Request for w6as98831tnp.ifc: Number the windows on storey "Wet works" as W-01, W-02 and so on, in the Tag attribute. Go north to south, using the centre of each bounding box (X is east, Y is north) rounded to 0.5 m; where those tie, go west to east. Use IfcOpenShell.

First a look at what the model holds.

```python
import ifcopenshell
import ifcopenshell.util.element
import ifcopenshell.util.placement

model = ifcopenshell.open("w6as98831tnp.ifc")
print(model.schema)
storey = next(s for s in model.by_type("IfcBuildingStorey") if s.Name == "Wet works")
windows = [e for e in ifcopenshell.util.element.get_decomposition(storey) if e.is_a("IfcWindow")]
for e in sorted(windows, key=lambda e: e.id()):
    origin = ifcopenshell.util.placement.get_local_placement(e.ObjectPlacement)[:3, 3]
    print(e.id(), e.Tag, e.Name, origin.round(2) + 0.0, sep=" | ")
```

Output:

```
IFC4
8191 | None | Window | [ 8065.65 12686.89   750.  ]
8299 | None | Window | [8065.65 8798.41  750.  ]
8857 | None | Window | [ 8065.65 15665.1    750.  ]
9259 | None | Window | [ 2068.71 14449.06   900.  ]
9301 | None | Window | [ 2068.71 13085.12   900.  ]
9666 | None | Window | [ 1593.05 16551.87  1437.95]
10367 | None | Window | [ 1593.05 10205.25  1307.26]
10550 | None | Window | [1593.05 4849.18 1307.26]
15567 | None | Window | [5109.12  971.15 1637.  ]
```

```python
import ifcopenshell
import ifcopenshell.geom
import ifcopenshell.util.element
import ifcopenshell.util.shape

model = ifcopenshell.open("w6as98831tnp.ifc")
settings = ifcopenshell.geom.settings()
settings.set("use-world-coords", True)


def centre(element):
    shape = ifcopenshell.geom.create_shape(settings, element)
    return ifcopenshell.util.shape.get_bbox_centroid(shape.geometry)


storey = next(s for s in model.by_type("IfcBuildingStorey") if s.Name == "Wet works")
windows = [e for e in ifcopenshell.util.element.get_decomposition(storey) if e.is_a("IfcWindow")]

# Insertion points can sit at a corner or the storey origin, so sort by the geometry (in metres).
centres = {e: centre(e) for e in windows}
windows.sort(key=lambda e: (-round(centres[e][1] / 0.5), centres[e][0]))

for i, e in enumerate(windows, start=1):
    number = f"W-{i:02d}"
    e.Tag = number
    print(e.id(), number)

model.write("w6as98831tnp-out.ifc")
```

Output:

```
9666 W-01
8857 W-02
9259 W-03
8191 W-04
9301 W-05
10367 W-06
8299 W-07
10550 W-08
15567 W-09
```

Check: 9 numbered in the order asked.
